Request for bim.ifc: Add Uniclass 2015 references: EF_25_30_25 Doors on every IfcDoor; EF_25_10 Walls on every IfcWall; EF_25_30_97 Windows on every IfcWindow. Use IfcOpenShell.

First a look at what the model holds.

```python
import ifcopenshell

model = ifcopenshell.open("bim.ifc")
print(model.schema)
print("classifications:", [c.Name for c in model.by_type("IfcClassification")])
for ifc_class in ("IfcDoor", "IfcRoof", "IfcStair", "IfcWall", "IfcWindow"):
    print(ifc_class, len(model.by_type(ifc_class)))
```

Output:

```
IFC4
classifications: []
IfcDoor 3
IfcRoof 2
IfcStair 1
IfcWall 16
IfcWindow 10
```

```python
import ifcopenshell
import ifcopenshell.api.classification

model = ifcopenshell.open("bim.ifc")

system = ifcopenshell.api.classification.add_classification(model, classification="Uniclass 2015")

codes = {
    "IfcDoor": ("EF_25_30_25", "Doors"),
    "IfcWall": ("EF_25_10", "Walls"),
    "IfcWindow": ("EF_25_30_97", "Windows"),
}
for ifc_class, (code, name) in codes.items():
    products = model.by_type(ifc_class)
    ifcopenshell.api.classification.add_reference(
        model, products=products, classification=system, identification=code, name=name
    )
    print(code, len(products))

model.write("bim-out.ifc")
```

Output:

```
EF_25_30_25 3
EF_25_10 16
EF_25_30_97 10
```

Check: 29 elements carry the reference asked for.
